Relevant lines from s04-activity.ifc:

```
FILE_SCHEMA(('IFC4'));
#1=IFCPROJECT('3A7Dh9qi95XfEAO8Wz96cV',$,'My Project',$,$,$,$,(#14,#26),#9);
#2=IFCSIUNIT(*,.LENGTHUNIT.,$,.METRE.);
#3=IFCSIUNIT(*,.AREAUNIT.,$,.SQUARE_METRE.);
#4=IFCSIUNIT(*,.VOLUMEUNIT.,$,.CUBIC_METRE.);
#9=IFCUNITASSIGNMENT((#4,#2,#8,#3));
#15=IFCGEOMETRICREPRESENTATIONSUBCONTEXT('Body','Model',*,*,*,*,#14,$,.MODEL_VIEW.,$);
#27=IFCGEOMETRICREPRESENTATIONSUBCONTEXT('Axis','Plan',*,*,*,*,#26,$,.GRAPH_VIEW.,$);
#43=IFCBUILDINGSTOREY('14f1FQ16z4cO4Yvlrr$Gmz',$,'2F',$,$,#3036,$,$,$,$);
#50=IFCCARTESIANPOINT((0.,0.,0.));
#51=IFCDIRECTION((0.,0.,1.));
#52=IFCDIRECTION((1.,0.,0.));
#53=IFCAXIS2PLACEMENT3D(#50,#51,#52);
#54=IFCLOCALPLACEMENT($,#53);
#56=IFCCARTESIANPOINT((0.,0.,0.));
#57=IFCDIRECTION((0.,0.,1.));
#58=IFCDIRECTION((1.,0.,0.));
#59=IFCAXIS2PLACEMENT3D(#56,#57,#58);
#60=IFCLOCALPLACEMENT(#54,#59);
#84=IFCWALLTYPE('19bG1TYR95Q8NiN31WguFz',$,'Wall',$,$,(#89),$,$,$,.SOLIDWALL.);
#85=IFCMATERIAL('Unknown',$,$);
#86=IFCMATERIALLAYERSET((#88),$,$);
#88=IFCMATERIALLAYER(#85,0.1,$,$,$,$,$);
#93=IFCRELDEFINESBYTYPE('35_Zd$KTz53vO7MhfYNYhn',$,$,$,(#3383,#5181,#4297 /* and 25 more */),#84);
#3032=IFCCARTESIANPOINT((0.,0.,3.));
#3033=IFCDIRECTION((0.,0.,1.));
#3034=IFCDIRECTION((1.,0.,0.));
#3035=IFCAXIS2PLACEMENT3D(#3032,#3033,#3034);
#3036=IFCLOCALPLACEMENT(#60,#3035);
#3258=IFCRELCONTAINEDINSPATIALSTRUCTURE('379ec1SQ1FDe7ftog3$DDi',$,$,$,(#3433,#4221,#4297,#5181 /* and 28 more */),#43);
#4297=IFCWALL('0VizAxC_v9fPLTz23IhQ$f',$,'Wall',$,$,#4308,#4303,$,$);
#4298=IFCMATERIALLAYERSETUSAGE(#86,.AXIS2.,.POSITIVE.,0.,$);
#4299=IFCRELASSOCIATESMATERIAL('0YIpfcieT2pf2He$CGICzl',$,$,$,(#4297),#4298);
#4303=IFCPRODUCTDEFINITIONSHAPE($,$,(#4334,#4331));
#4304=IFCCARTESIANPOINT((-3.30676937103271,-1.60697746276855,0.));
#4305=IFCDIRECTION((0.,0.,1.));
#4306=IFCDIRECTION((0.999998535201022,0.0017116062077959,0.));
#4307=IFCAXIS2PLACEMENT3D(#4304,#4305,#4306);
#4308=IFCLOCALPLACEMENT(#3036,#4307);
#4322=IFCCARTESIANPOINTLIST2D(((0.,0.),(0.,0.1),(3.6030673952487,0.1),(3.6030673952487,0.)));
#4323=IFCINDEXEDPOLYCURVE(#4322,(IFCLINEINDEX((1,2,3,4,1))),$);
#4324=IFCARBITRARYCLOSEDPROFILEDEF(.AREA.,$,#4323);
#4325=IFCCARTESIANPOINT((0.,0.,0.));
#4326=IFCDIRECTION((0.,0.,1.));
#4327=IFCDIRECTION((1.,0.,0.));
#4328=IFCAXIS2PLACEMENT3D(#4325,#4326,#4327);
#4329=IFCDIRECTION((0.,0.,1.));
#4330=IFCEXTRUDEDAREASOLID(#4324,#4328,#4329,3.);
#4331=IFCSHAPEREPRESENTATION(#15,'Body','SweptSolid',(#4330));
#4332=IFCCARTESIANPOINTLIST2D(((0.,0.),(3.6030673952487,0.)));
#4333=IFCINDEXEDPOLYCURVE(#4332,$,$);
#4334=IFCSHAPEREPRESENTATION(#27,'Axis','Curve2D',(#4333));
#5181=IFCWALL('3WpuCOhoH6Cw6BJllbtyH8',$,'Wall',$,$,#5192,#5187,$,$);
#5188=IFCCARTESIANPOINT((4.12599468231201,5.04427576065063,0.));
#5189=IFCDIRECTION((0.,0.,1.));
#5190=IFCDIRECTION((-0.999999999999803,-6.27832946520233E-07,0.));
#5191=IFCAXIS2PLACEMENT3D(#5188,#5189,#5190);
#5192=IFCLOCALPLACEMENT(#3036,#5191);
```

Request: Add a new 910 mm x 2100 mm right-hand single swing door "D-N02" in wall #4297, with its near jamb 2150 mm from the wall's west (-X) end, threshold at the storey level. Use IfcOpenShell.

```python
import numpy as np
import ifcopenshell
import ifcopenshell.api.feature
import ifcopenshell.api.geometry
import ifcopenshell.api.root
import ifcopenshell.api.spatial
import ifcopenshell.geom
import ifcopenshell.util.element
import ifcopenshell.util.placement
import ifcopenshell.util.representation
import ifcopenshell.util.shape
import ifcopenshell.util.unit

model = ifcopenshell.open("s04-activity.ifc")
unit_scale = ifcopenshell.util.unit.calculate_unit_scale(model)
settings = ifcopenshell.geom.settings()


def volume(element):
    """Net volume in cubic metres, openings subtracted."""
    shape = ifcopenshell.geom.create_shape(settings, element)
    return ifcopenshell.util.shape.get_volume(shape.geometry)


wall = model.by_guid("0VizAxC_v9fPLTz23IhQ$f")
storey = ifcopenshell.util.element.get_container(wall, ifc_class="IfcBuildingStorey")
context = ifcopenshell.util.representation.get_context(model, "Model", "Body", "MODEL_VIEW")
before = volume(wall)

width, height, from_end, sill = 0.91, 2.1, 2.15, 0.0  # metres

# The wall runs along its own X axis, and the end named is its -X end.
wall_shape = ifcopenshell.geom.create_shape(settings, wall)
x, y, z = ifcopenshell.util.shape.get_vertices(wall_shape.geometry).T
start = x.min() + from_end
face, thickness = float(y.min()), float(y.max() - y.min())
wall_matrix = ifcopenshell.util.placement.get_local_placement(wall.ObjectPlacement)
level = ifcopenshell.util.placement.get_local_placement(storey.ObjectPlacement)[2, 3]


def in_wall(x, y):
    """Placement at x, y metres in the wall's axes, at sill height."""
    matrix = wall_matrix.copy()
    matrix[:, 3] = wall_matrix @ np.array([x / unit_scale, y / unit_scale, 0.0, 1.0])
    matrix[2, 3] = level + sill / unit_scale
    return matrix


# Opening: a box that overshoots both wall faces by 50 mm.
opening = ifcopenshell.api.root.create_entity(model, ifc_class="IfcOpeningElement", predefined_type="OPENING")
box = ifcopenshell.api.geometry.add_wall_representation(
    model, context=context, length=width, height=height, thickness=thickness + 0.1
)
ifcopenshell.api.geometry.assign_representation(model, product=opening, representation=box)
ifcopenshell.api.geometry.edit_object_placement(model, product=opening, matrix=in_wall(start, face - 0.05), is_si=False)
ifcopenshell.api.feature.add_feature(model, feature=opening, element=wall)

door = ifcopenshell.api.root.create_entity(model, ifc_class="IfcDoor", name="D-N02", predefined_type="DOOR")
door.OverallWidth, door.OverallHeight = width / unit_scale, height / unit_scale
door.OperationType = "SINGLE_SWING_RIGHT"
body = ifcopenshell.api.geometry.add_door_representation(
    model,
    context=context,
    overall_width=door.OverallWidth,
    overall_height=door.OverallHeight,
    operation_type="SINGLE_SWING_RIGHT",
    lining_properties={"LiningDepth": thickness / unit_scale, "ThresholdDepth": thickness / unit_scale},
)
ifcopenshell.api.geometry.assign_representation(model, product=door, representation=body)
ifcopenshell.api.spatial.assign_container(model, products=[door], relating_structure=storey)
ifcopenshell.api.feature.add_filling(model, opening=opening, element=door)

# The lining spans the wall, so the door starts at the wall face.
ifcopenshell.api.geometry.edit_object_placement(model, product=door, matrix=in_wall(start, face), is_si=False)

after = volume(wall)

print(f"wall volume {before:.3f} -> {after:.3f} m3")

model.write("s04-activity-out.ifc")
```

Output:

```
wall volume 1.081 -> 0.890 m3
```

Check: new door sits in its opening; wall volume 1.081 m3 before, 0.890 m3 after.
